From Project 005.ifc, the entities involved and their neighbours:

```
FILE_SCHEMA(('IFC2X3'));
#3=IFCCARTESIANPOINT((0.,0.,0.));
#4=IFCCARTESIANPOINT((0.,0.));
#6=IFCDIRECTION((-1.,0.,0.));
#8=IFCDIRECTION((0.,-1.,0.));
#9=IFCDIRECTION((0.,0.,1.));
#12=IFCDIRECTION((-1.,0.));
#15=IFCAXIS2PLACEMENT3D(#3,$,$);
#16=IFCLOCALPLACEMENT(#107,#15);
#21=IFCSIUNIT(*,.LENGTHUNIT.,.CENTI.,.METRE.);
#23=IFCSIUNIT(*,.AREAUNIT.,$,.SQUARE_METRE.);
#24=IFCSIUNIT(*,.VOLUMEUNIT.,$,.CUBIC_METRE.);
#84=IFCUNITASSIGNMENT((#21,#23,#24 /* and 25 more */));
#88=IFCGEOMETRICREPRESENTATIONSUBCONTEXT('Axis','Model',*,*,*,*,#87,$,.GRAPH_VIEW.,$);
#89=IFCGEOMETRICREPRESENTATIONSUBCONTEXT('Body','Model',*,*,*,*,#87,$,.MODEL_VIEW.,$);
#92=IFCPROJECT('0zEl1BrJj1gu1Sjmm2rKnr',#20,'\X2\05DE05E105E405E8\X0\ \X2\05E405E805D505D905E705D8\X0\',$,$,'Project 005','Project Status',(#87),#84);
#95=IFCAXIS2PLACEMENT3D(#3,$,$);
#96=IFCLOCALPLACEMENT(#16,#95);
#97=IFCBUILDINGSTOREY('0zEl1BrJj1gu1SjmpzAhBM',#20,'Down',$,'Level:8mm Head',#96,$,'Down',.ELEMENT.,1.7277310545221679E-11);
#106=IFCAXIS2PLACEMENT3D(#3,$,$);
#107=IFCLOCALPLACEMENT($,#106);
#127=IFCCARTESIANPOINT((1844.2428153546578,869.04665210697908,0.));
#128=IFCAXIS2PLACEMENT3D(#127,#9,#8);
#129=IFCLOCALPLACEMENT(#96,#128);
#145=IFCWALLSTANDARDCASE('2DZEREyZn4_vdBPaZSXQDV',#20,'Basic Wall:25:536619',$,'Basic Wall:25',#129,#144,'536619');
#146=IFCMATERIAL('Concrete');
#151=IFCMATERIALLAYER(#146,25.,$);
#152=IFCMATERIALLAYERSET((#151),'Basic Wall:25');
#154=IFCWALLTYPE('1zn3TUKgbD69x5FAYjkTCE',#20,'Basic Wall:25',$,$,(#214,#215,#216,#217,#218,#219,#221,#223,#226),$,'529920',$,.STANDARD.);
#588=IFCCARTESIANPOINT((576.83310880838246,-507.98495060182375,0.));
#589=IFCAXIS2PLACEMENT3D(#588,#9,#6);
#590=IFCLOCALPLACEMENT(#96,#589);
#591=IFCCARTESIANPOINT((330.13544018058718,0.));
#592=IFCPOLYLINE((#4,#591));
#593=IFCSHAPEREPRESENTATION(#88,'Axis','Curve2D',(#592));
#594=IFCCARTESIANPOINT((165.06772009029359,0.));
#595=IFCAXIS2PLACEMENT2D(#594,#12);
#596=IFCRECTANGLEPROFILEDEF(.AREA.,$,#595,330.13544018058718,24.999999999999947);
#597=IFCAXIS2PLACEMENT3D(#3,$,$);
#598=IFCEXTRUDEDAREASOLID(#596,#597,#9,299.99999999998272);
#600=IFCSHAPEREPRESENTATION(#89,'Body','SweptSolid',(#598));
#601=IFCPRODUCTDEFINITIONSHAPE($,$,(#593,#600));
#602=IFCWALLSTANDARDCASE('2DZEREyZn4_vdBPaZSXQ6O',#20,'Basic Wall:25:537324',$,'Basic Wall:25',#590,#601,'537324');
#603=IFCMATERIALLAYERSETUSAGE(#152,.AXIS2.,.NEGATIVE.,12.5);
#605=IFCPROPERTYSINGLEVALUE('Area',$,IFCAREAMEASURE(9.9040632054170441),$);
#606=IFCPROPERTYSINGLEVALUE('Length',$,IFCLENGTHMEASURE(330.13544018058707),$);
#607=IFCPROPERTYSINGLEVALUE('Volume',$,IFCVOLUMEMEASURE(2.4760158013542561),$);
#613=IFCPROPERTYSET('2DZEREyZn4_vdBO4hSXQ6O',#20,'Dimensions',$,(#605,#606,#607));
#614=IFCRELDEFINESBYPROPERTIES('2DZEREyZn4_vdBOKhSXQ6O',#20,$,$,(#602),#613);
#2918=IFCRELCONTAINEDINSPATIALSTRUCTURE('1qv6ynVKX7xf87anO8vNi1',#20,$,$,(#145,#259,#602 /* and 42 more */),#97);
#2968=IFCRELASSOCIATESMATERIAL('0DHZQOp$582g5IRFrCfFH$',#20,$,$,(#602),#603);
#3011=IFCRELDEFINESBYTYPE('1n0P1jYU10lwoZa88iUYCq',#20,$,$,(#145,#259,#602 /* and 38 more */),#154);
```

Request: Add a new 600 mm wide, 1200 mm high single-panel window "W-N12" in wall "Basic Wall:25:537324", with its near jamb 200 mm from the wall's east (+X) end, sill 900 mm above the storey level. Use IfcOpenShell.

```python
import numpy as np
import ifcopenshell
import ifcopenshell.api.feature
import ifcopenshell.api.geometry
import ifcopenshell.api.pset
import ifcopenshell.api.root
import ifcopenshell.api.spatial
import ifcopenshell.api.type
import ifcopenshell.geom
import ifcopenshell.util.element
import ifcopenshell.util.placement
import ifcopenshell.util.representation
import ifcopenshell.util.shape
import ifcopenshell.util.unit

model = ifcopenshell.open("Project 005.ifc")
unit_scale = ifcopenshell.util.unit.calculate_unit_scale(model)
area_scale = ifcopenshell.util.unit.calculate_unit_scale(model, "AREAUNIT")
volume_scale = ifcopenshell.util.unit.calculate_unit_scale(model, "VOLUMEUNIT")
settings = ifcopenshell.geom.settings()


def volume(element):
    """Net volume in cubic metres, openings subtracted."""
    shape = ifcopenshell.geom.create_shape(settings, element)
    return ifcopenshell.util.shape.get_volume(shape.geometry)


wall = model.by_id(602)
storey = ifcopenshell.util.element.get_container(wall, ifc_class="IfcBuildingStorey")
context = ifcopenshell.util.representation.get_context(model, "Model", "Body", "MODEL_VIEW")
before = volume(wall)

width, height, from_end, sill = 0.6, 1.2, 0.2, 0.9  # metres

# The wall runs along its own X axis, and the end named is its -X end.
wall_shape = ifcopenshell.geom.create_shape(settings, wall)
x, y, z = ifcopenshell.util.shape.get_vertices(wall_shape.geometry).T
start = x.min() + from_end
face, thickness = float(y.min()), float(y.max() - y.min())
wall_matrix = ifcopenshell.util.placement.get_local_placement(wall.ObjectPlacement)
level = ifcopenshell.util.placement.get_local_placement(storey.ObjectPlacement)[2, 3]


def in_wall(x, y):
    """Placement at x, y metres in the wall's axes, at sill height."""
    matrix = wall_matrix.copy()
    matrix[:, 3] = wall_matrix @ np.array([x / unit_scale, y / unit_scale, 0.0, 1.0])
    matrix[2, 3] = level + sill / unit_scale
    return matrix


# Opening: a box that overshoots both wall faces by 50 mm.
opening = ifcopenshell.api.root.create_entity(model, ifc_class="IfcOpeningElement")
box = ifcopenshell.api.geometry.add_wall_representation(
    model, context=context, length=width, height=height, thickness=thickness + 0.1
)
ifcopenshell.api.geometry.assign_representation(model, product=opening, representation=box)
ifcopenshell.api.geometry.edit_object_placement(model, product=opening, matrix=in_wall(start, face - 0.05), is_si=False)
ifcopenshell.api.feature.add_feature(model, feature=opening, element=wall)

window = ifcopenshell.api.root.create_entity(model, ifc_class="IfcWindow", name="W-N12")
window.OverallWidth, window.OverallHeight = width / unit_scale, height / unit_scale
body = ifcopenshell.api.geometry.add_window_representation(
    model,
    context=context,
    overall_width=window.OverallWidth,
    overall_height=window.OverallHeight,
    partition_type="SINGLE_PANEL",
)
ifcopenshell.api.geometry.assign_representation(model, product=window, representation=body)
ifcopenshell.api.spatial.assign_container(model, products=[window], relating_structure=storey)
fills = ifcopenshell.api.feature.add_filling(model, opening=opening, element=window)
fills.OwnerHistory = window.OwnerHistory  # required in IFC2X3

# IFC2X3 keeps the operation on the window style.
style = ifcopenshell.api.root.create_entity(model, ifc_class="IfcWindowStyle", name="W-N12")
style.OperationType, style.ConstructionType = "SINGLE_PANEL", "NOTDEFINED"
style.ParameterTakesPrecedence = style.Sizeable = False
ifcopenshell.api.type.assign_type(model, related_objects=[window], relating_type=style)

# Centre the window in the wall's thickness.
ifcopenshell.api.geometry.edit_object_placement(model, product=window, matrix=in_wall(start, face), is_si=False)
window_shape = ifcopenshell.geom.create_shape(settings, window)
depth = ifcopenshell.util.shape.get_vertices(window_shape.geometry)[:, 1]
offset = face + thickness / 2 - (depth.min() + depth.max()) / 2
ifcopenshell.api.geometry.edit_object_placement(model, product=window, matrix=in_wall(start, offset), is_si=False)

after = volume(wall)

# Update the wall's stored quantities.
pset = model.by_id(ifcopenshell.util.element.get_pset(wall, "Dimensions", should_inherit=False)["id"])
ifcopenshell.api.pset.edit_pset(model, pset=pset, properties={
    "Area": model.create_entity("IfcAreaMeasure", after / thickness / area_scale),
    "Volume": model.create_entity("IfcVolumeMeasure", after / volume_scale),
})

print(f"wall volume {before:.3f} -> {after:.3f} m3")

model.write("Project 005_rev.ifc")
```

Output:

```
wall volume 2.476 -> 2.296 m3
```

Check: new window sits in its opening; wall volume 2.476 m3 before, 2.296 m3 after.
